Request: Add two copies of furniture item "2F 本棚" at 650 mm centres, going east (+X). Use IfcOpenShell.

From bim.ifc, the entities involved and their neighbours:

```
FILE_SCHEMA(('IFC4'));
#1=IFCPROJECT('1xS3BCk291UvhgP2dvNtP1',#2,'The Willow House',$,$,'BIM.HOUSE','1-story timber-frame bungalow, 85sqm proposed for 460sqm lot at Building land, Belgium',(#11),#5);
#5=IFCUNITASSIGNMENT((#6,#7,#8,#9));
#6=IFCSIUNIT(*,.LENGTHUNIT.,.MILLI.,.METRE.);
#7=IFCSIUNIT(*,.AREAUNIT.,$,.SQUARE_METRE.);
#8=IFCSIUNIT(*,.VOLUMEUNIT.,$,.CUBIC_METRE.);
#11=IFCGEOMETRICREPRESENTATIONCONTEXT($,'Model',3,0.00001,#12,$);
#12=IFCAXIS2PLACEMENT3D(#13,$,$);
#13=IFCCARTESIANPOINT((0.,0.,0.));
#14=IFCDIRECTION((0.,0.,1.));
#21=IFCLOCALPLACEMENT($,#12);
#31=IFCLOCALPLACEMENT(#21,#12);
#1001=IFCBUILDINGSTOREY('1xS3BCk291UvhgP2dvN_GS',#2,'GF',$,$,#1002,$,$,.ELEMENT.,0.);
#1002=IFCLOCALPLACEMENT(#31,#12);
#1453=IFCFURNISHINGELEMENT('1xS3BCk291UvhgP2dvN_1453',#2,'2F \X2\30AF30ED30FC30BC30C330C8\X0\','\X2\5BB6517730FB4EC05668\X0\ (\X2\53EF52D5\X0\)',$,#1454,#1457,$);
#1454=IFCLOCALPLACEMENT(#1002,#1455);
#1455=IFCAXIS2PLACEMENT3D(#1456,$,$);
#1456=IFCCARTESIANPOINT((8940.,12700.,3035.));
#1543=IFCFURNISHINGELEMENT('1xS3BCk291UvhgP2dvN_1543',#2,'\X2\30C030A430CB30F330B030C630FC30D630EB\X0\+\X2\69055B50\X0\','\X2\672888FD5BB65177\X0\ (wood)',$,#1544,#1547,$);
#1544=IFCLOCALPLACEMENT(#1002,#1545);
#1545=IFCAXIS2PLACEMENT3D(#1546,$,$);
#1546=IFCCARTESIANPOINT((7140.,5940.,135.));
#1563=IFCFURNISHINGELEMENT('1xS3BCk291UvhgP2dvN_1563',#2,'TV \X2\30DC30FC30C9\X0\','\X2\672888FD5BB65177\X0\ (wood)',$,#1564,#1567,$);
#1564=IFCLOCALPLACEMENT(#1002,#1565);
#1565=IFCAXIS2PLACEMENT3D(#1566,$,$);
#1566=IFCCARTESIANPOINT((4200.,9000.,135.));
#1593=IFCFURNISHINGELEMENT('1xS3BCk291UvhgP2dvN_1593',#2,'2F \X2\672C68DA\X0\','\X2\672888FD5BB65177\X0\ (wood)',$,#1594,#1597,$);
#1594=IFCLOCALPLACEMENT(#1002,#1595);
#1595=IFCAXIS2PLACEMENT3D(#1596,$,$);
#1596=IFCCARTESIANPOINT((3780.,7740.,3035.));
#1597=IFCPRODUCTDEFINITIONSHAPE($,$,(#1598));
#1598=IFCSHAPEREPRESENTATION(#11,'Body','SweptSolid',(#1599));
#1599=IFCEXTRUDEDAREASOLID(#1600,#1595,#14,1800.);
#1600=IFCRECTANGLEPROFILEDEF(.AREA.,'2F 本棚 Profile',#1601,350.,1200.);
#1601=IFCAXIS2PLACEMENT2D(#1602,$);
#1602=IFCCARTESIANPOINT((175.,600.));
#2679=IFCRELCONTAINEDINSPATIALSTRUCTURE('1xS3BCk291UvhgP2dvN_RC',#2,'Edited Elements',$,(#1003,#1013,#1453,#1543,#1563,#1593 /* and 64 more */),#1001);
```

```python
import numpy as np
import ifcopenshell
import ifcopenshell.api.geometry
import ifcopenshell.api.root
import ifcopenshell.util.element
import ifcopenshell.util.placement
import ifcopenshell.util.unit

model = ifcopenshell.open("bim.ifc")
unit_scale = ifcopenshell.util.unit.calculate_unit_scale(model)


def reuse_history(source, copy):
    """copy_class also copies each property set's owner history, people and application; keep the originals."""
    for rel in copy.IsDefinedBy:
        if rel.is_a("IfcRelDefinesByProperties") and (history := rel.RelatingPropertyDefinition.OwnerHistory):
            rel.RelatingPropertyDefinition.OwnerHistory = source.OwnerHistory
            ifcopenshell.util.element.remove_deep2(model, history)


source = model.by_guid("1xS3BCk291UvhgP2dvN_1593")
base = ifcopenshell.util.placement.get_local_placement(source.ObjectPlacement)
step = np.array([1.0, 0.0, 0.0]) * 0.65 / unit_scale

for i in range(1, 3):
    copy = ifcopenshell.api.root.copy_class(model, product=source)
    copy.Representation = ifcopenshell.util.element.copy_deep(
        model, source.Representation, exclude=["IfcGeometricRepresentationContext", "IfcRepresentationMap"]
    )
    reuse_history(source, copy)
    matrix = base.copy()
    matrix[:3, 3] += i * step
    print("added at", matrix[:3, 3].round(3) + 0.0)
    ifcopenshell.api.geometry.edit_object_placement(model, product=copy, matrix=matrix, is_si=False)

model.write("bim_updated.ifc")
```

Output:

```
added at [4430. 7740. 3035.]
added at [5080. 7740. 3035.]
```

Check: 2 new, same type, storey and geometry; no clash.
